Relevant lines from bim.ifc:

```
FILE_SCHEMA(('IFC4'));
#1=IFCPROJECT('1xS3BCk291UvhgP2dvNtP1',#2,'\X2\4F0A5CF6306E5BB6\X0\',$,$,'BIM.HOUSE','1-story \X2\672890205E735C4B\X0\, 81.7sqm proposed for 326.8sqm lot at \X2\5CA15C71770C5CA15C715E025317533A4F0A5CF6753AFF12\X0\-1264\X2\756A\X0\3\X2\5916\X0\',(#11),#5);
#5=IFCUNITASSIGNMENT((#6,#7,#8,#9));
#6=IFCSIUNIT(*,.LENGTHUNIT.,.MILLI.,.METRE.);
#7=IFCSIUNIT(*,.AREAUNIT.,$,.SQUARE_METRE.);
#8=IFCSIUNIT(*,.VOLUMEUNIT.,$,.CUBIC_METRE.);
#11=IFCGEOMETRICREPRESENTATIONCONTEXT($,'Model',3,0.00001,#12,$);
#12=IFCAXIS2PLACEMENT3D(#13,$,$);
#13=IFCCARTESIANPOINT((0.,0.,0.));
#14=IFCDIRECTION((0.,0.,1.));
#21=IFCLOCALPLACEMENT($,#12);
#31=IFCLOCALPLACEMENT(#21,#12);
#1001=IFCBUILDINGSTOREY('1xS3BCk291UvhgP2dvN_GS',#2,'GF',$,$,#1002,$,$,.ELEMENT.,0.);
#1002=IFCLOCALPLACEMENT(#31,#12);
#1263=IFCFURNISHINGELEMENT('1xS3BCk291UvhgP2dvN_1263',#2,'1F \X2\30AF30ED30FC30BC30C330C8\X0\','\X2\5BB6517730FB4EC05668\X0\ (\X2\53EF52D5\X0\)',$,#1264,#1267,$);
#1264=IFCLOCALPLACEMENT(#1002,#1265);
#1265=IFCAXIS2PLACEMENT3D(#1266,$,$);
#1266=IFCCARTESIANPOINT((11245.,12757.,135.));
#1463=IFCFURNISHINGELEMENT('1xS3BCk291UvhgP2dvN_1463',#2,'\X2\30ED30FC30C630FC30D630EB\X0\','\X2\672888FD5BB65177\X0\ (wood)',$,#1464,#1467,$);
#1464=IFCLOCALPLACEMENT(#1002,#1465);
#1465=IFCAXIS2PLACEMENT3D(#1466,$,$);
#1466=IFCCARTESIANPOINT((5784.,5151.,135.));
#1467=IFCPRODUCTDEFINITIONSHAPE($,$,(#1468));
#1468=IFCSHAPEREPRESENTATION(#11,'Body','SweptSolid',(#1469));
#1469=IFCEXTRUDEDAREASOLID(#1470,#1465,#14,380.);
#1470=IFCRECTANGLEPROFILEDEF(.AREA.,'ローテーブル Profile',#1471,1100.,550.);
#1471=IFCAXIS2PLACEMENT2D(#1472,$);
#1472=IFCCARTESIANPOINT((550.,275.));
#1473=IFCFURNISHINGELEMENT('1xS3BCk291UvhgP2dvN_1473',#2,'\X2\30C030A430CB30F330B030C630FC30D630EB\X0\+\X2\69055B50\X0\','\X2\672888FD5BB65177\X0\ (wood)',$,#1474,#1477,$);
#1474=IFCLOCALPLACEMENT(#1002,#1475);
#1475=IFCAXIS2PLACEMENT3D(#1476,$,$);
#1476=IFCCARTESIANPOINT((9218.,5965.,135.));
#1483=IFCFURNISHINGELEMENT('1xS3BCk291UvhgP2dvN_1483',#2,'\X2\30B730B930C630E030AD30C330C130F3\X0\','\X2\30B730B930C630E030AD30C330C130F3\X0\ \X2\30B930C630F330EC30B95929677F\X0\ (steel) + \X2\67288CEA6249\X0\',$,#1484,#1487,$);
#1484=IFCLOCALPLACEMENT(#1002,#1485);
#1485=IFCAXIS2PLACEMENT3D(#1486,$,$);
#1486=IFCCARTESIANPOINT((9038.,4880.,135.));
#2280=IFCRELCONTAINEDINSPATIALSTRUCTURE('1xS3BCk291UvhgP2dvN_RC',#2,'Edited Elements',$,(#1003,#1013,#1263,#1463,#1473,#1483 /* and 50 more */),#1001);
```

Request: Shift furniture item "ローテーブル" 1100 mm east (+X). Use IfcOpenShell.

```python
import ifcopenshell
import ifcopenshell.api.geometry
import ifcopenshell.util.placement
import ifcopenshell.util.unit

model = ifcopenshell.open("bim.ifc")
unit_scale = ifcopenshell.util.unit.calculate_unit_scale(model)

item = model.by_guid("1xS3BCk291UvhgP2dvN_1463")
matrix = ifcopenshell.util.placement.get_local_placement(item.ObjectPlacement)
matrix[0, 3] += 1.1 / unit_scale
ifcopenshell.api.geometry.edit_object_placement(model, product=item, matrix=matrix, is_si=False)

print(ifcopenshell.util.placement.get_local_placement(item.ObjectPlacement).round(3) + 0.0)

model.write("bim_updated.ifc")
```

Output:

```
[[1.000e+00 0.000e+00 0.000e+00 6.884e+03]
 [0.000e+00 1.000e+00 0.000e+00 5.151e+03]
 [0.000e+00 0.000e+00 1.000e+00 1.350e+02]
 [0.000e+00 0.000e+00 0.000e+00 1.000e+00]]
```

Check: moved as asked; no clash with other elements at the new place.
